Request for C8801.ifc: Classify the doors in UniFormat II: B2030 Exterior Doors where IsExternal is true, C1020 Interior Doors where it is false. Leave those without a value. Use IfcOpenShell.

First a look at what the model holds.

```python
import ifcopenshell
import ifcopenshell.util.element

model = ifcopenshell.open("C8801.ifc")
print(model.schema)
print("classifications:", [c.Name for c in model.by_type("IfcClassification")])
values = [ifcopenshell.util.element.get_pset(e, "Pset_DoorCommon", "IsExternal") for e in model.by_type("IfcDoor")]
for value in (True, False, None):
    print("IsExternal", value, values.count(value))
```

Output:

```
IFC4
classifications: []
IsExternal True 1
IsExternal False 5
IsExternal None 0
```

```python
import ifcopenshell
import ifcopenshell.api.classification
import ifcopenshell.util.element

model = ifcopenshell.open("C8801.ifc")

system = ifcopenshell.api.classification.add_classification(model, classification="UniFormat II")

doors = model.by_type("IfcDoor")
external = {e: ifcopenshell.util.element.get_pset(e, "Pset_DoorCommon", "IsExternal") for e in doors}
for flag, code, name in ((True, "B2030", "Exterior Doors"), (False, "C1020", "Interior Doors")):
    products = [e for e in doors if external[e] is flag]
    ifcopenshell.api.classification.add_reference(
        model, products=products, classification=system, identification=code, name=name
    )
    print(code, len(products))

model.write("C8801_updated.ifc")
```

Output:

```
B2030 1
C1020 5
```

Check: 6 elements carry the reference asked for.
